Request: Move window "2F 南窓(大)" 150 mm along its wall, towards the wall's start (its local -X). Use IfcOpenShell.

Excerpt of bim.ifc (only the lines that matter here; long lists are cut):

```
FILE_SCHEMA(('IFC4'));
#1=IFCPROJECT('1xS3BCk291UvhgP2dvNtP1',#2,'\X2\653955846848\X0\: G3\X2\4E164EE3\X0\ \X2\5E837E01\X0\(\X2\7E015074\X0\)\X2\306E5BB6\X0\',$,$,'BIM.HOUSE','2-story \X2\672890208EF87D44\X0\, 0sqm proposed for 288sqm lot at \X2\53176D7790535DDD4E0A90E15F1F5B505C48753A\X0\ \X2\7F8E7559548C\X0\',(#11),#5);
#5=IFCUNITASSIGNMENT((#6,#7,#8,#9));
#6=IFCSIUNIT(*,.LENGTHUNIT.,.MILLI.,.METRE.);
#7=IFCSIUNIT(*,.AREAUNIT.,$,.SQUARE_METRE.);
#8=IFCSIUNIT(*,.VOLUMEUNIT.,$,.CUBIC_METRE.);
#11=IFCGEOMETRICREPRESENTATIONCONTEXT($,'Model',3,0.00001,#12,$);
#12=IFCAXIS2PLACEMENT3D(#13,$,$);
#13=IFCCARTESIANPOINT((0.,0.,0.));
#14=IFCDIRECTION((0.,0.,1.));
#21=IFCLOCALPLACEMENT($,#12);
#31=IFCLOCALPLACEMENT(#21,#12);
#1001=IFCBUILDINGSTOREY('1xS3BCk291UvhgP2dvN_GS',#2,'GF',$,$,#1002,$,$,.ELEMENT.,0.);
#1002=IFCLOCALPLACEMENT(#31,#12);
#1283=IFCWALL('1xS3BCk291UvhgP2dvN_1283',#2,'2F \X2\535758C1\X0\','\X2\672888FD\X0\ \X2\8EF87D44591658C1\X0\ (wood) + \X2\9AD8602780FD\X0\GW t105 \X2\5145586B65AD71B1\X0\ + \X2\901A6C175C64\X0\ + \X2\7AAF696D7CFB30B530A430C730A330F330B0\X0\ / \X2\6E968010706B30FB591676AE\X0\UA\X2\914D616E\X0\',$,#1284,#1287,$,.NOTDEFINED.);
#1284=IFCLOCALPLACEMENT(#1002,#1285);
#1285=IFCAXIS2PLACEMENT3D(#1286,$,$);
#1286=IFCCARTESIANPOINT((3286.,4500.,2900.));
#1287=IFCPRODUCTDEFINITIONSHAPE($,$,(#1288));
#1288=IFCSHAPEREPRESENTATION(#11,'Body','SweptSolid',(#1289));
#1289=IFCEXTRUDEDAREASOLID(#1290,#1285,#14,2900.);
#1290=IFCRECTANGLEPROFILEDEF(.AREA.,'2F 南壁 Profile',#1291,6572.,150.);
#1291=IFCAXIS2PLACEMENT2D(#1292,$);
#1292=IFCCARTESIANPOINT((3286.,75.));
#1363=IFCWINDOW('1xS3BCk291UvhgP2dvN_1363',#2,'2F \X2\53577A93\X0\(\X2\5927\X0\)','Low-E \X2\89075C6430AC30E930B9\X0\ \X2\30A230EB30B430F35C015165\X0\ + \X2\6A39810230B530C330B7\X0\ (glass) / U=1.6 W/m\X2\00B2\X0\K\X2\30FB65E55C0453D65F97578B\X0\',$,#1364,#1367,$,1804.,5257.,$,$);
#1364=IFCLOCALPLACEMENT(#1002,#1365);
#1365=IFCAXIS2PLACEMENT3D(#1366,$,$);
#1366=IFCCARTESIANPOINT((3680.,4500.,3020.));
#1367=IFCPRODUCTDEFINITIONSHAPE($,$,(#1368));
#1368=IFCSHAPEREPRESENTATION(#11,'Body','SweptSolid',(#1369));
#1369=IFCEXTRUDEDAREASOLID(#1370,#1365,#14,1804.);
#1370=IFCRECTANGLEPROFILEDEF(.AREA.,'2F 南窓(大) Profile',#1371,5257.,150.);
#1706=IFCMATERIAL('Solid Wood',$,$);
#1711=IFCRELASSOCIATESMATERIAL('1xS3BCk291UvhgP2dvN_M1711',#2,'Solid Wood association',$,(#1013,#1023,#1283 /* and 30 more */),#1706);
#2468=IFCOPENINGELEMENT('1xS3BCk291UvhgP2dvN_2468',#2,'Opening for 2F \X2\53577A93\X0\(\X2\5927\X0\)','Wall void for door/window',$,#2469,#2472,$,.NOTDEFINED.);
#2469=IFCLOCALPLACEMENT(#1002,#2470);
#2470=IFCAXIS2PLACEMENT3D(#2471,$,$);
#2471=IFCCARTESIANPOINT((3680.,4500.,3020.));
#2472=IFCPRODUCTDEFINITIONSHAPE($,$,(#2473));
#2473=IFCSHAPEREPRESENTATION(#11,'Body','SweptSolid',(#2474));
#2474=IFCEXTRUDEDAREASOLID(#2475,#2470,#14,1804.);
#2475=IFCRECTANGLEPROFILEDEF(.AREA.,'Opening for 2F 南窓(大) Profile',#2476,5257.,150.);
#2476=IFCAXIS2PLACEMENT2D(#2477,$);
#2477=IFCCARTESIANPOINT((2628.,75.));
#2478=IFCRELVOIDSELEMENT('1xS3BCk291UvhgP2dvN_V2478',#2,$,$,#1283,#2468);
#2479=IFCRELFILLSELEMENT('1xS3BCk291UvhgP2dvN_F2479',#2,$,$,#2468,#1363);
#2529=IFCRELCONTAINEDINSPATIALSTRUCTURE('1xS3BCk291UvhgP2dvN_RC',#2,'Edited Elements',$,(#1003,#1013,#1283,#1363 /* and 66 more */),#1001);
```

```python
import ifcopenshell
import ifcopenshell.api.geometry
import ifcopenshell.util.placement
import ifcopenshell.util.unit

model = ifcopenshell.open("bim.ifc")
unit_scale = ifcopenshell.util.unit.calculate_unit_scale(model)

window = model.by_guid("1xS3BCk291UvhgP2dvN_1363")
opening = window.FillsVoids[0].RelatingOpeningElement
wall = opening.VoidsElements[0].RelatingBuildingElement

wall_matrix = ifcopenshell.util.placement.get_local_placement(wall.ObjectPlacement)
shift = wall_matrix[:3, 0] * -0.15 / unit_scale
before = ifcopenshell.util.placement.get_local_placement(window.ObjectPlacement)[:3, 3].copy()

# The window is not placed relative to its opening, so move both.
for product in (opening, window):
    matrix = ifcopenshell.util.placement.get_local_placement(product.ObjectPlacement)
    matrix[:3, 3] += shift
    ifcopenshell.api.geometry.edit_object_placement(model, product=product, matrix=matrix, is_si=False)

after = ifcopenshell.util.placement.get_local_placement(window.ObjectPlacement)[:3, 3]
print("window moved by", (after - before).round(3) + 0.0)

model.write("bim_v2.ifc")
```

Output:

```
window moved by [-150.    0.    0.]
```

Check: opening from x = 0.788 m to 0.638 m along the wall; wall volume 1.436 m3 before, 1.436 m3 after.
